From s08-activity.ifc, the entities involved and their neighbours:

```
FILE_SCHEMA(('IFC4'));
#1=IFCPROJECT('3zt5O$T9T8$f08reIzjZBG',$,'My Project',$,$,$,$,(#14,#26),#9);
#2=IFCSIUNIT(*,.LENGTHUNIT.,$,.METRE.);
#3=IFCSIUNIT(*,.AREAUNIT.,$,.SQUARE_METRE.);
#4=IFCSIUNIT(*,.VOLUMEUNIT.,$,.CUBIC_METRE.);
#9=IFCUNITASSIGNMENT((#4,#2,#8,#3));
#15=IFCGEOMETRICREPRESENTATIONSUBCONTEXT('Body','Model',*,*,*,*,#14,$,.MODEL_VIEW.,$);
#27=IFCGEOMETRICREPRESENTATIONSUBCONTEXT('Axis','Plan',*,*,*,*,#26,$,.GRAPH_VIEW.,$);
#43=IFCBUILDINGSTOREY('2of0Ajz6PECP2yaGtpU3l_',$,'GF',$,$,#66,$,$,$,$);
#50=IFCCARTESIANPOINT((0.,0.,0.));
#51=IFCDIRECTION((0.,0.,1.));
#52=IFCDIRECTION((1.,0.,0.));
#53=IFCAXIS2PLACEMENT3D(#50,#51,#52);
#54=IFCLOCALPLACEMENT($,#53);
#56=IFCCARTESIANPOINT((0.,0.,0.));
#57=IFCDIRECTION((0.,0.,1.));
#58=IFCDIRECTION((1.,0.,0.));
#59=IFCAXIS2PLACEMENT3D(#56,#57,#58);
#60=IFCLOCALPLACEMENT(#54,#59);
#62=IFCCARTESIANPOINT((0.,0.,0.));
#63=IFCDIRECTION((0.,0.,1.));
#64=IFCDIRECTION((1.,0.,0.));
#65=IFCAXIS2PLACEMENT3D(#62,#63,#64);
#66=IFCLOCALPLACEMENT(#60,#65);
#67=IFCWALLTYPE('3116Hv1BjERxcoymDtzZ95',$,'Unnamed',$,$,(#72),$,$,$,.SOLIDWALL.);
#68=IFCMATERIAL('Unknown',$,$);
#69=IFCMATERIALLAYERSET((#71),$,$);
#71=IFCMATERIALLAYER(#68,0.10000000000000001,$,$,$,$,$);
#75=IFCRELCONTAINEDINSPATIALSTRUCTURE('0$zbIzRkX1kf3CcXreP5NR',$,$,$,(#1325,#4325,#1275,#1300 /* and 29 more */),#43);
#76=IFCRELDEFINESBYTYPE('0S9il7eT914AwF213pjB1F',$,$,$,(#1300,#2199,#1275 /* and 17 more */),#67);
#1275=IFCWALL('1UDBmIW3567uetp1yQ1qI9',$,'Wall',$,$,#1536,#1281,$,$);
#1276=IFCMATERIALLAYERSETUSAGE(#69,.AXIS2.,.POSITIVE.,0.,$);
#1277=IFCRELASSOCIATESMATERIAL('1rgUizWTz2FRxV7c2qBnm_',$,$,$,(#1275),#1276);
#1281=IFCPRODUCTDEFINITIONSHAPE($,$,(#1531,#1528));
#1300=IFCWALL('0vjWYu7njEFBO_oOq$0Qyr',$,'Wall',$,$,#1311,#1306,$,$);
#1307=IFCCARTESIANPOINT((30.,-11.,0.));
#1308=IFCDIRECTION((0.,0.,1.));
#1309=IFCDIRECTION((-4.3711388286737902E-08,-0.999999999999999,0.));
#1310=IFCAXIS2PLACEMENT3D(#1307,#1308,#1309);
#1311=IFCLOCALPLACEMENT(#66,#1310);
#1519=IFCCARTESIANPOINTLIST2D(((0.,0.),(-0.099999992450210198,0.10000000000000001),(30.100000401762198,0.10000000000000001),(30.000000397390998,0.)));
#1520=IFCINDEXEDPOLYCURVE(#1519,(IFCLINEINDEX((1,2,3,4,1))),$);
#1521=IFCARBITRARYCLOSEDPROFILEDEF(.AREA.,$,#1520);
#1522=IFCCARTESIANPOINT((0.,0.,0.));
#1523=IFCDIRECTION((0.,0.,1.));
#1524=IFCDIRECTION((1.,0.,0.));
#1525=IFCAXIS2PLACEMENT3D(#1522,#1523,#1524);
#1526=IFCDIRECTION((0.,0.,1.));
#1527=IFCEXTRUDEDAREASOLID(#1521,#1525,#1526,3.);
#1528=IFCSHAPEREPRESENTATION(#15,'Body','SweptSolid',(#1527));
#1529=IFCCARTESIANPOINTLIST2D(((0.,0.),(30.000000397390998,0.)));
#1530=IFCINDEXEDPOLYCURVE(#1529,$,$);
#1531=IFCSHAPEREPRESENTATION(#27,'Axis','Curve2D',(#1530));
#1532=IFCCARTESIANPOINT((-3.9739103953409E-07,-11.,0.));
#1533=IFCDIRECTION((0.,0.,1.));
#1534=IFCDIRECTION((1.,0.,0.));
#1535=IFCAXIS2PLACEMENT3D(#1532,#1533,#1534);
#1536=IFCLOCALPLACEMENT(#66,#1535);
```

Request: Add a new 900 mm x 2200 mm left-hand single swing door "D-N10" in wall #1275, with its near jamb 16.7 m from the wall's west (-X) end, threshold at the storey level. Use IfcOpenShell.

```python
import numpy as np
import ifcopenshell
import ifcopenshell.api.feature
import ifcopenshell.api.geometry
import ifcopenshell.api.root
import ifcopenshell.api.spatial
import ifcopenshell.geom
import ifcopenshell.util.element
import ifcopenshell.util.placement
import ifcopenshell.util.representation
import ifcopenshell.util.shape
import ifcopenshell.util.unit

model = ifcopenshell.open("s08-activity.ifc")
unit_scale = ifcopenshell.util.unit.calculate_unit_scale(model)
settings = ifcopenshell.geom.settings()


def volume(element):
    """Net volume in cubic metres, openings subtracted."""
    shape = ifcopenshell.geom.create_shape(settings, element)
    return ifcopenshell.util.shape.get_volume(shape.geometry)


wall = model.by_guid("1UDBmIW3567uetp1yQ1qI9")
storey = ifcopenshell.util.element.get_container(wall, ifc_class="IfcBuildingStorey")
context = ifcopenshell.util.representation.get_context(model, "Model", "Body", "MODEL_VIEW")
before = volume(wall)

width, height, from_end, sill = 0.9, 2.2, 16.7, 0.0  # metres

# The wall runs along its own X axis, and the end named is its -X end.
wall_shape = ifcopenshell.geom.create_shape(settings, wall)
x, y, z = ifcopenshell.util.shape.get_vertices(wall_shape.geometry).T
start = x.min() + from_end
face, thickness = float(y.min()), float(y.max() - y.min())
wall_matrix = ifcopenshell.util.placement.get_local_placement(wall.ObjectPlacement)
level = ifcopenshell.util.placement.get_local_placement(storey.ObjectPlacement)[2, 3]


def in_wall(x, y):
    """Placement at x, y metres in the wall's axes, at sill height."""
    matrix = wall_matrix.copy()
    matrix[:, 3] = wall_matrix @ np.array([x / unit_scale, y / unit_scale, 0.0, 1.0])
    matrix[2, 3] = level + sill / unit_scale
    return matrix


# Opening: a box that overshoots both wall faces by 50 mm.
opening = ifcopenshell.api.root.create_entity(model, ifc_class="IfcOpeningElement", predefined_type="OPENING")
box = ifcopenshell.api.geometry.add_wall_representation(
    model, context=context, length=width, height=height, thickness=thickness + 0.1
)
ifcopenshell.api.geometry.assign_representation(model, product=opening, representation=box)
ifcopenshell.api.geometry.edit_object_placement(model, product=opening, matrix=in_wall(start, face - 0.05), is_si=False)
ifcopenshell.api.feature.add_feature(model, feature=opening, element=wall)

door = ifcopenshell.api.root.create_entity(model, ifc_class="IfcDoor", name="D-N10", predefined_type="DOOR")
door.OverallWidth, door.OverallHeight = width / unit_scale, height / unit_scale
door.OperationType = "SINGLE_SWING_LEFT"
body = ifcopenshell.api.geometry.add_door_representation(
    model,
    context=context,
    overall_width=door.OverallWidth,
    overall_height=door.OverallHeight,
    operation_type="SINGLE_SWING_LEFT",
    lining_properties={"LiningDepth": thickness / unit_scale, "ThresholdDepth": thickness / unit_scale},
)
ifcopenshell.api.geometry.assign_representation(model, product=door, representation=body)
ifcopenshell.api.spatial.assign_container(model, products=[door], relating_structure=storey)
ifcopenshell.api.feature.add_filling(model, opening=opening, element=door)

# The lining spans the wall, so the door starts at the wall face.
ifcopenshell.api.geometry.edit_object_placement(model, product=door, matrix=in_wall(start, face), is_si=False)

after = volume(wall)

print(f"wall volume {before:.3f} -> {after:.3f} m3")

model.write("s08-activity_updated.ifc")
```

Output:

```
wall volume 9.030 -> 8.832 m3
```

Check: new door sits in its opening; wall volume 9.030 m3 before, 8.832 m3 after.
